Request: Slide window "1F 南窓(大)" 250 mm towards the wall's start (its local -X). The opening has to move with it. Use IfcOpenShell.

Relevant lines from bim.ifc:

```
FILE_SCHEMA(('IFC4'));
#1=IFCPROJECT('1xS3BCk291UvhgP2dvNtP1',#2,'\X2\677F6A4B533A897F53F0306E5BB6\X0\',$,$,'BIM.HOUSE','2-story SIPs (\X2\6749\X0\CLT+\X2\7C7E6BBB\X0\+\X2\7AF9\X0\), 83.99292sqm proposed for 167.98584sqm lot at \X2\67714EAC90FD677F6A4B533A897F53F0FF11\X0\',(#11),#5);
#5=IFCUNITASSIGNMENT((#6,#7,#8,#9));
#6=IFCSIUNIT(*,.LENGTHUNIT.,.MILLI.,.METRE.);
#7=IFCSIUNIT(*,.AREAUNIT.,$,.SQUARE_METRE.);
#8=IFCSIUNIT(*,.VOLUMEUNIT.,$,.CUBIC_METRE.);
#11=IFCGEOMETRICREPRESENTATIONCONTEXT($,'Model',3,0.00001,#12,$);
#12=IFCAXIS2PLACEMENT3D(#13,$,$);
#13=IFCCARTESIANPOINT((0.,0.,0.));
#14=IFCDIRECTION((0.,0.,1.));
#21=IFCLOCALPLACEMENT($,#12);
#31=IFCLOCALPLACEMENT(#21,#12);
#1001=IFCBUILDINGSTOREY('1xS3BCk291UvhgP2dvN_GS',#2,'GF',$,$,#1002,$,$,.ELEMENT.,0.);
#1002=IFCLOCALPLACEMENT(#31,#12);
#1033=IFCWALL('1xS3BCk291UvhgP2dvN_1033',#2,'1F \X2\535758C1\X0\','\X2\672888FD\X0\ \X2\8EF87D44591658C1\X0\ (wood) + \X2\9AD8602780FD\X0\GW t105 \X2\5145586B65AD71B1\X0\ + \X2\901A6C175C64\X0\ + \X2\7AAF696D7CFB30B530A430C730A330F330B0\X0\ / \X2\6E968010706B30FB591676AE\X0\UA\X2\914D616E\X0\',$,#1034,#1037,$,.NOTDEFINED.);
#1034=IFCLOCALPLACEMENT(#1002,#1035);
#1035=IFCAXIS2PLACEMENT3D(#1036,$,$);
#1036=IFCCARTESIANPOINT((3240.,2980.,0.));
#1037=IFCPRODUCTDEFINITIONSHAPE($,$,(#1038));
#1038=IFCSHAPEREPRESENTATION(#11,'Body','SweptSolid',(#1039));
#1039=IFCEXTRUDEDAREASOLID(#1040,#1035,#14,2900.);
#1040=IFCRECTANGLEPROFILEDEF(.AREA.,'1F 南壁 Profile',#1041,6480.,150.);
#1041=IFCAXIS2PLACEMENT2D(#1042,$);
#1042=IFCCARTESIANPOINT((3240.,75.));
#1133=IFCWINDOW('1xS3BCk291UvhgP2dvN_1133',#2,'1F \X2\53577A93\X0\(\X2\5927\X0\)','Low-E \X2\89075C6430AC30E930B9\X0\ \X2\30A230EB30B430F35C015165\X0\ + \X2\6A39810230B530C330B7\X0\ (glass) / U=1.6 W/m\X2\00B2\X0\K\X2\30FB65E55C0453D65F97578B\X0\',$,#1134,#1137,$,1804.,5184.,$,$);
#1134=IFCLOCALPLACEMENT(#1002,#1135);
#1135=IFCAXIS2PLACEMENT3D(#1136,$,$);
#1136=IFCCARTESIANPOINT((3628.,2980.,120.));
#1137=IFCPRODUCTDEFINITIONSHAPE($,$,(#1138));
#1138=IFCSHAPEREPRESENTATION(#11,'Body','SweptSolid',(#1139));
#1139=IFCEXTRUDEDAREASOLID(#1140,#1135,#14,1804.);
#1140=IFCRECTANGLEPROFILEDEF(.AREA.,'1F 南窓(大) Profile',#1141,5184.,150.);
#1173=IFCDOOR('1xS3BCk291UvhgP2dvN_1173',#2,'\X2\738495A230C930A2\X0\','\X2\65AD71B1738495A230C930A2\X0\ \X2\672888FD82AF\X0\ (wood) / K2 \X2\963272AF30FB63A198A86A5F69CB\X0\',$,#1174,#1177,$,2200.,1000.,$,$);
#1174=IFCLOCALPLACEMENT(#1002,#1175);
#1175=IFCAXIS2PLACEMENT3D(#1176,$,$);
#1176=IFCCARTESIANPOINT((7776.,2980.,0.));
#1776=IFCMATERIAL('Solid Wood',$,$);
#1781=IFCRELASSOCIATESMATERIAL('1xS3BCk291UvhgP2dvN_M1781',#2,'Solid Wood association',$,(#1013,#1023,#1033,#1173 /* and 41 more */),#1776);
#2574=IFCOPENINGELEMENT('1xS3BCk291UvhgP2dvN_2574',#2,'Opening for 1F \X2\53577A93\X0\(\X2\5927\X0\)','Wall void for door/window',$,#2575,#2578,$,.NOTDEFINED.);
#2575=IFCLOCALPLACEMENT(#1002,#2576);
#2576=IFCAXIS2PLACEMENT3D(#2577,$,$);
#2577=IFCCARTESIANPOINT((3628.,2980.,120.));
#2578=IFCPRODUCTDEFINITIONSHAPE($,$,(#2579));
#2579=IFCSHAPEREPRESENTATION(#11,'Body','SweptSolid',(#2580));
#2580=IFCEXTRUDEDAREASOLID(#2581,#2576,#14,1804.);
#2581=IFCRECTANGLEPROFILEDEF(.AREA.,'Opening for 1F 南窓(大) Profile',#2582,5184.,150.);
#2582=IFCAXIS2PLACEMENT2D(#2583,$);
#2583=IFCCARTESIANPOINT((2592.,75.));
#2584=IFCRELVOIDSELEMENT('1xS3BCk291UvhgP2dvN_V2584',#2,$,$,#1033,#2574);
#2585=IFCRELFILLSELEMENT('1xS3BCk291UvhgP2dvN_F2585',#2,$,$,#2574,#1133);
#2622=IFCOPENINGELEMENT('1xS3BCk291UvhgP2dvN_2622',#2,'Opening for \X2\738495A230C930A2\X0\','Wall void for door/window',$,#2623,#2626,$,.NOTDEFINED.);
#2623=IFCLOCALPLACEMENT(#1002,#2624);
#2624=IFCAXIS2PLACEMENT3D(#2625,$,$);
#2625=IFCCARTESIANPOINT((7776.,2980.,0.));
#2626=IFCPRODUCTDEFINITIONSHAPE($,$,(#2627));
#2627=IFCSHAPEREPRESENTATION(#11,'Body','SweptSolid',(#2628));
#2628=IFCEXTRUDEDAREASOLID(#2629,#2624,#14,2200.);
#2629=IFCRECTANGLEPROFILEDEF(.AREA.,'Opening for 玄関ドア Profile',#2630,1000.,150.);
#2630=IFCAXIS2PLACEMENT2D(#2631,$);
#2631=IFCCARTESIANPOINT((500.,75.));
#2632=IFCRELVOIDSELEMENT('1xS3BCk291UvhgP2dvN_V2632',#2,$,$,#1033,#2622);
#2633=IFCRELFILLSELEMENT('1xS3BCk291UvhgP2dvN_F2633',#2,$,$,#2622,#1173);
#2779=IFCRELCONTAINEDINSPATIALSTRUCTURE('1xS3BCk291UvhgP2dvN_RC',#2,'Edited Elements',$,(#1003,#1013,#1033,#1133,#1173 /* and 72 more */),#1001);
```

```python
import ifcopenshell
import ifcopenshell.api.geometry
import ifcopenshell.util.placement

model = ifcopenshell.open("bim.ifc")

window = model.by_id(1133)
opening = window.FillsVoids[0].RelatingOpeningElement
wall = opening.VoidsElements[0].RelatingBuildingElement

wall_matrix = ifcopenshell.util.placement.get_local_placement(wall.ObjectPlacement)
shift = wall_matrix[:3, 0] * -250.0
before = ifcopenshell.util.placement.get_local_placement(window.ObjectPlacement)[:3, 3].copy()

# The window is not placed relative to its opening, so move both.
for product in (opening, window):
    matrix = ifcopenshell.util.placement.get_local_placement(product.ObjectPlacement)
    matrix[:3, 3] += shift
    ifcopenshell.api.geometry.edit_object_placement(model, product=product, matrix=matrix, is_si=False)

after = ifcopenshell.util.placement.get_local_placement(window.ObjectPlacement)[:3, 3]
print("window moved by", (after - before).round(3) + 0.0)

model.write("bim_edited.ifc")
```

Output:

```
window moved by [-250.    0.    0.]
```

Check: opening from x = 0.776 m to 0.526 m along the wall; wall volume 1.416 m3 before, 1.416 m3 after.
